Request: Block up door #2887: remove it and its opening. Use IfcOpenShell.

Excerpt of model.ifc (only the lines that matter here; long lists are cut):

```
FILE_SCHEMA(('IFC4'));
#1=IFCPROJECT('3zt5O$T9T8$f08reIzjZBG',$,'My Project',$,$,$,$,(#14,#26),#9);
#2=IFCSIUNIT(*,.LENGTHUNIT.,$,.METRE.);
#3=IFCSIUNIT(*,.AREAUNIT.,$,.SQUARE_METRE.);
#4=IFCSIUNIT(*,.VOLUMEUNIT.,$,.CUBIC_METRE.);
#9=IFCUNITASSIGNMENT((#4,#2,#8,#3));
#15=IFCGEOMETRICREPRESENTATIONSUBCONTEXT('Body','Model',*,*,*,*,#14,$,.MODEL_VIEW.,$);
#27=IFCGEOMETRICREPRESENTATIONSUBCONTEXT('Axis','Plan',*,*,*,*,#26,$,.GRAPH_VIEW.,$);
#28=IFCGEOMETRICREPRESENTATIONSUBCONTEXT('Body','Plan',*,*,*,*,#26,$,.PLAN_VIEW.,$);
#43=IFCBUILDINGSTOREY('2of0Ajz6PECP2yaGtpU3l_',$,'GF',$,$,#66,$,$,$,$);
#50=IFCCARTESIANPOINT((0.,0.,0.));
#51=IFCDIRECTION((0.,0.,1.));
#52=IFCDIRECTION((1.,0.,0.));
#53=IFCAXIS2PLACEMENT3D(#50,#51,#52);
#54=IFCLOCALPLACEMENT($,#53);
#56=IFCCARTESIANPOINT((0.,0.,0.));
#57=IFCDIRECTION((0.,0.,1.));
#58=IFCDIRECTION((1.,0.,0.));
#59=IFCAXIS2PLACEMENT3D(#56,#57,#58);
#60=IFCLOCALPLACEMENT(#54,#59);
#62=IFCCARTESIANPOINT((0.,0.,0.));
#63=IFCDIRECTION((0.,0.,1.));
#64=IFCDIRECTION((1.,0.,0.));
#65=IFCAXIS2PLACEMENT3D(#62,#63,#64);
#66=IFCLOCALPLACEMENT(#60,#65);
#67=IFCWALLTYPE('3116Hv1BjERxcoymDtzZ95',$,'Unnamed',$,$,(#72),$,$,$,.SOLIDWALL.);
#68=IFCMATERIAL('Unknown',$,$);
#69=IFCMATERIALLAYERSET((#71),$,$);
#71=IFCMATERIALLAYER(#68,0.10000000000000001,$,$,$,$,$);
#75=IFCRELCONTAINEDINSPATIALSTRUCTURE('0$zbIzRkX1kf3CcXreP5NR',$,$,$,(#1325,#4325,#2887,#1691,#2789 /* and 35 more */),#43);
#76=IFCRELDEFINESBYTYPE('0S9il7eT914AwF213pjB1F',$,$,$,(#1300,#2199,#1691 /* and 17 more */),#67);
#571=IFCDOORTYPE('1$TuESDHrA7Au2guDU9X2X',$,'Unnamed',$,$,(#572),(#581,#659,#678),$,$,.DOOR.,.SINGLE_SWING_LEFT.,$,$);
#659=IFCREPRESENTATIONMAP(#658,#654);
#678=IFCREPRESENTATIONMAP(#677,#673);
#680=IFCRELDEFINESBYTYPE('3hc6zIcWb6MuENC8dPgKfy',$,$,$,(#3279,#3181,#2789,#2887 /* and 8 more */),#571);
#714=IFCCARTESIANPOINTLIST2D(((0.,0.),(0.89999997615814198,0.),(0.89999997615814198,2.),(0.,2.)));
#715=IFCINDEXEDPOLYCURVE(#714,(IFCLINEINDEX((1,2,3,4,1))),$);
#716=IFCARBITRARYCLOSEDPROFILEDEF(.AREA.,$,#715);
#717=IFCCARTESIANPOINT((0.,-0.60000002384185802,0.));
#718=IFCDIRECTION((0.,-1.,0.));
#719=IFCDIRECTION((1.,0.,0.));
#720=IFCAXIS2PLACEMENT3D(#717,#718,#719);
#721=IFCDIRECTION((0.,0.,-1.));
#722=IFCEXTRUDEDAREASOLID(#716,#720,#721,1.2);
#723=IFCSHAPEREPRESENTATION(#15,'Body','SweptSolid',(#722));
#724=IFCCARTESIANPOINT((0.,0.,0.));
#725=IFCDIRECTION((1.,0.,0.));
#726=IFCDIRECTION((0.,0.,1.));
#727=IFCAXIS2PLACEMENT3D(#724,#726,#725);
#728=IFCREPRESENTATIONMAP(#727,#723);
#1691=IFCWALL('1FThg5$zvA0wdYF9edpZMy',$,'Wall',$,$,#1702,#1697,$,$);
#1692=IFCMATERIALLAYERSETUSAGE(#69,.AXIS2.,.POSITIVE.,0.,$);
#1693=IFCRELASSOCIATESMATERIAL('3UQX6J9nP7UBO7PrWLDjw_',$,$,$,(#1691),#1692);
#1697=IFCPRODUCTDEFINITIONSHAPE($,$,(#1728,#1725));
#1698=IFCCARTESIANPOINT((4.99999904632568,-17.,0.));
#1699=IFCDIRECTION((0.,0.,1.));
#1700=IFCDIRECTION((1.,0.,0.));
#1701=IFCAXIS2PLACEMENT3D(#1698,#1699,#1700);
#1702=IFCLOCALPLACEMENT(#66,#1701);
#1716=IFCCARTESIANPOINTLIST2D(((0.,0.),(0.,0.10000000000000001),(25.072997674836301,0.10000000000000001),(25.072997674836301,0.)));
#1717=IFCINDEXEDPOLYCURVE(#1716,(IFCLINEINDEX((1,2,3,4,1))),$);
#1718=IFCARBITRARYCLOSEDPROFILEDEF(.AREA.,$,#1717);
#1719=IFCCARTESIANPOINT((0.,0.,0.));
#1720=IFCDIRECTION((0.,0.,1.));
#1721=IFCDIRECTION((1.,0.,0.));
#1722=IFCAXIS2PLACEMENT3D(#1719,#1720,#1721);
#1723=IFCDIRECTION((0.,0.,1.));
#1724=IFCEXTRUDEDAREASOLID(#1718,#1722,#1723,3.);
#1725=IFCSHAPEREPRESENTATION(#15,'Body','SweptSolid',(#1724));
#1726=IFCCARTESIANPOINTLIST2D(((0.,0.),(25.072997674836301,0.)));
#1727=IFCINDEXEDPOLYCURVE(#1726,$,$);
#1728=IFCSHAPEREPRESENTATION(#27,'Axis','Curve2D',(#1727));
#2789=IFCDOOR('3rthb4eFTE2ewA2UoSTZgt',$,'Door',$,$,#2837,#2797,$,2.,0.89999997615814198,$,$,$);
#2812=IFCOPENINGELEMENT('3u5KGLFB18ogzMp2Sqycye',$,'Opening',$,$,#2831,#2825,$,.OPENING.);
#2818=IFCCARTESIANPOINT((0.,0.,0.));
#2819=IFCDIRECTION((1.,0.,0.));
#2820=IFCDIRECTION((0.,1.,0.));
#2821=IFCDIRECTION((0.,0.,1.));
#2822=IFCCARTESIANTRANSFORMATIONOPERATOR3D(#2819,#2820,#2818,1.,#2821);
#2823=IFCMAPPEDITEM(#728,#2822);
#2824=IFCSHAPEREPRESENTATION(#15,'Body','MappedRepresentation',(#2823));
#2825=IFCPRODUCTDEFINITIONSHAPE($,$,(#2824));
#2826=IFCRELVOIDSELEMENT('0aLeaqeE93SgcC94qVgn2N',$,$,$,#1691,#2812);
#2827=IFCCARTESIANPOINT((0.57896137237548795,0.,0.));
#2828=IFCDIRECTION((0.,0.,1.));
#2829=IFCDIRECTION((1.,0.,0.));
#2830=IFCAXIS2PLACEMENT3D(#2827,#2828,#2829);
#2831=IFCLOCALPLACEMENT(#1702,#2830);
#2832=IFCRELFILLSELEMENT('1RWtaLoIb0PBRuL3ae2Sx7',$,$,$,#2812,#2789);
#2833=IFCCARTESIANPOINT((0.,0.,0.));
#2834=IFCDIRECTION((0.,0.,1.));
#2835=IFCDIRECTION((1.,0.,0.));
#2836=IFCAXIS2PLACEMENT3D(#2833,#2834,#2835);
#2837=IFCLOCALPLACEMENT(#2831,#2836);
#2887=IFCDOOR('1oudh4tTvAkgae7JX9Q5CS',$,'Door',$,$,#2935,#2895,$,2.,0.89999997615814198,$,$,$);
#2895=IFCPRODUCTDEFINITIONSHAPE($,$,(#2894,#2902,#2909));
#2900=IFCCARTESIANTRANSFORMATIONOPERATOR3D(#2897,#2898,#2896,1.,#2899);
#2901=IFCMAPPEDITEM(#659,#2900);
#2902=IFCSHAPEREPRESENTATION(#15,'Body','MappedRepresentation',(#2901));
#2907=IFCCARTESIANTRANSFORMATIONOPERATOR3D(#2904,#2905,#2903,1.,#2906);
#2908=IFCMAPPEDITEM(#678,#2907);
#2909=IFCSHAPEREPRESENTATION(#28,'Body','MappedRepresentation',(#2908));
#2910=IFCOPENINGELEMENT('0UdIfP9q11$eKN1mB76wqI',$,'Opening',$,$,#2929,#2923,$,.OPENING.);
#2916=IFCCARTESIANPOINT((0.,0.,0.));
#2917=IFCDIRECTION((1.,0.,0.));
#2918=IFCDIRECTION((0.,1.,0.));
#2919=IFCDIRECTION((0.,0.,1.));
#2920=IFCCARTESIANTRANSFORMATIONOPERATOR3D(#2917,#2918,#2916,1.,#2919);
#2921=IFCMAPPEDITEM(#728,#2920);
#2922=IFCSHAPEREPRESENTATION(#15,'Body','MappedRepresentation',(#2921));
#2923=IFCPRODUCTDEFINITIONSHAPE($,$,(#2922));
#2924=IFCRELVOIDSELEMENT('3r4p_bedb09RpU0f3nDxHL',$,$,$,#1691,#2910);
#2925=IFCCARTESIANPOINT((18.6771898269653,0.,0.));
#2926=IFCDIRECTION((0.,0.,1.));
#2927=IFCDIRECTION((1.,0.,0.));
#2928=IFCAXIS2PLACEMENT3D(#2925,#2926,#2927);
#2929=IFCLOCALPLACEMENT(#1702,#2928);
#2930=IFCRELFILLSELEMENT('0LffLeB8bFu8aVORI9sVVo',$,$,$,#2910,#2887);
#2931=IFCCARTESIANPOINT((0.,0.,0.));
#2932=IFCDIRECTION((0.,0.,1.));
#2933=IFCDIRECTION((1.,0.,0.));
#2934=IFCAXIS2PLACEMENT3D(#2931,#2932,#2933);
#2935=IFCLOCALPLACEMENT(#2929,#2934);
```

```python
import ifcopenshell
import ifcopenshell.api.feature
import ifcopenshell.api.root
import ifcopenshell.geom
import ifcopenshell.util.shape

model = ifcopenshell.open("model.ifc")
settings = ifcopenshell.geom.settings()


def volume(element):
    """Net volume in cubic metres, openings subtracted."""
    shape = ifcopenshell.geom.create_shape(settings, element)
    return ifcopenshell.util.shape.get_volume(shape.geometry)


door = model.by_guid("1oudh4tTvAkgae7JX9Q5CS")
opening = door.FillsVoids[0].RelatingOpeningElement
wall = opening.VoidsElements[0].RelatingBuildingElement
before = volume(wall)

ifcopenshell.api.root.remove_product(model, product=door)
ifcopenshell.api.feature.remove_feature(model, feature=opening)

after = volume(wall)

print(f"wall volume {before:.3f} -> {after:.3f} m3")

model.write("model_updated.ifc")
```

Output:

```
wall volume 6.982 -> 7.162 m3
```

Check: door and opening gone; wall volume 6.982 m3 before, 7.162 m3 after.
